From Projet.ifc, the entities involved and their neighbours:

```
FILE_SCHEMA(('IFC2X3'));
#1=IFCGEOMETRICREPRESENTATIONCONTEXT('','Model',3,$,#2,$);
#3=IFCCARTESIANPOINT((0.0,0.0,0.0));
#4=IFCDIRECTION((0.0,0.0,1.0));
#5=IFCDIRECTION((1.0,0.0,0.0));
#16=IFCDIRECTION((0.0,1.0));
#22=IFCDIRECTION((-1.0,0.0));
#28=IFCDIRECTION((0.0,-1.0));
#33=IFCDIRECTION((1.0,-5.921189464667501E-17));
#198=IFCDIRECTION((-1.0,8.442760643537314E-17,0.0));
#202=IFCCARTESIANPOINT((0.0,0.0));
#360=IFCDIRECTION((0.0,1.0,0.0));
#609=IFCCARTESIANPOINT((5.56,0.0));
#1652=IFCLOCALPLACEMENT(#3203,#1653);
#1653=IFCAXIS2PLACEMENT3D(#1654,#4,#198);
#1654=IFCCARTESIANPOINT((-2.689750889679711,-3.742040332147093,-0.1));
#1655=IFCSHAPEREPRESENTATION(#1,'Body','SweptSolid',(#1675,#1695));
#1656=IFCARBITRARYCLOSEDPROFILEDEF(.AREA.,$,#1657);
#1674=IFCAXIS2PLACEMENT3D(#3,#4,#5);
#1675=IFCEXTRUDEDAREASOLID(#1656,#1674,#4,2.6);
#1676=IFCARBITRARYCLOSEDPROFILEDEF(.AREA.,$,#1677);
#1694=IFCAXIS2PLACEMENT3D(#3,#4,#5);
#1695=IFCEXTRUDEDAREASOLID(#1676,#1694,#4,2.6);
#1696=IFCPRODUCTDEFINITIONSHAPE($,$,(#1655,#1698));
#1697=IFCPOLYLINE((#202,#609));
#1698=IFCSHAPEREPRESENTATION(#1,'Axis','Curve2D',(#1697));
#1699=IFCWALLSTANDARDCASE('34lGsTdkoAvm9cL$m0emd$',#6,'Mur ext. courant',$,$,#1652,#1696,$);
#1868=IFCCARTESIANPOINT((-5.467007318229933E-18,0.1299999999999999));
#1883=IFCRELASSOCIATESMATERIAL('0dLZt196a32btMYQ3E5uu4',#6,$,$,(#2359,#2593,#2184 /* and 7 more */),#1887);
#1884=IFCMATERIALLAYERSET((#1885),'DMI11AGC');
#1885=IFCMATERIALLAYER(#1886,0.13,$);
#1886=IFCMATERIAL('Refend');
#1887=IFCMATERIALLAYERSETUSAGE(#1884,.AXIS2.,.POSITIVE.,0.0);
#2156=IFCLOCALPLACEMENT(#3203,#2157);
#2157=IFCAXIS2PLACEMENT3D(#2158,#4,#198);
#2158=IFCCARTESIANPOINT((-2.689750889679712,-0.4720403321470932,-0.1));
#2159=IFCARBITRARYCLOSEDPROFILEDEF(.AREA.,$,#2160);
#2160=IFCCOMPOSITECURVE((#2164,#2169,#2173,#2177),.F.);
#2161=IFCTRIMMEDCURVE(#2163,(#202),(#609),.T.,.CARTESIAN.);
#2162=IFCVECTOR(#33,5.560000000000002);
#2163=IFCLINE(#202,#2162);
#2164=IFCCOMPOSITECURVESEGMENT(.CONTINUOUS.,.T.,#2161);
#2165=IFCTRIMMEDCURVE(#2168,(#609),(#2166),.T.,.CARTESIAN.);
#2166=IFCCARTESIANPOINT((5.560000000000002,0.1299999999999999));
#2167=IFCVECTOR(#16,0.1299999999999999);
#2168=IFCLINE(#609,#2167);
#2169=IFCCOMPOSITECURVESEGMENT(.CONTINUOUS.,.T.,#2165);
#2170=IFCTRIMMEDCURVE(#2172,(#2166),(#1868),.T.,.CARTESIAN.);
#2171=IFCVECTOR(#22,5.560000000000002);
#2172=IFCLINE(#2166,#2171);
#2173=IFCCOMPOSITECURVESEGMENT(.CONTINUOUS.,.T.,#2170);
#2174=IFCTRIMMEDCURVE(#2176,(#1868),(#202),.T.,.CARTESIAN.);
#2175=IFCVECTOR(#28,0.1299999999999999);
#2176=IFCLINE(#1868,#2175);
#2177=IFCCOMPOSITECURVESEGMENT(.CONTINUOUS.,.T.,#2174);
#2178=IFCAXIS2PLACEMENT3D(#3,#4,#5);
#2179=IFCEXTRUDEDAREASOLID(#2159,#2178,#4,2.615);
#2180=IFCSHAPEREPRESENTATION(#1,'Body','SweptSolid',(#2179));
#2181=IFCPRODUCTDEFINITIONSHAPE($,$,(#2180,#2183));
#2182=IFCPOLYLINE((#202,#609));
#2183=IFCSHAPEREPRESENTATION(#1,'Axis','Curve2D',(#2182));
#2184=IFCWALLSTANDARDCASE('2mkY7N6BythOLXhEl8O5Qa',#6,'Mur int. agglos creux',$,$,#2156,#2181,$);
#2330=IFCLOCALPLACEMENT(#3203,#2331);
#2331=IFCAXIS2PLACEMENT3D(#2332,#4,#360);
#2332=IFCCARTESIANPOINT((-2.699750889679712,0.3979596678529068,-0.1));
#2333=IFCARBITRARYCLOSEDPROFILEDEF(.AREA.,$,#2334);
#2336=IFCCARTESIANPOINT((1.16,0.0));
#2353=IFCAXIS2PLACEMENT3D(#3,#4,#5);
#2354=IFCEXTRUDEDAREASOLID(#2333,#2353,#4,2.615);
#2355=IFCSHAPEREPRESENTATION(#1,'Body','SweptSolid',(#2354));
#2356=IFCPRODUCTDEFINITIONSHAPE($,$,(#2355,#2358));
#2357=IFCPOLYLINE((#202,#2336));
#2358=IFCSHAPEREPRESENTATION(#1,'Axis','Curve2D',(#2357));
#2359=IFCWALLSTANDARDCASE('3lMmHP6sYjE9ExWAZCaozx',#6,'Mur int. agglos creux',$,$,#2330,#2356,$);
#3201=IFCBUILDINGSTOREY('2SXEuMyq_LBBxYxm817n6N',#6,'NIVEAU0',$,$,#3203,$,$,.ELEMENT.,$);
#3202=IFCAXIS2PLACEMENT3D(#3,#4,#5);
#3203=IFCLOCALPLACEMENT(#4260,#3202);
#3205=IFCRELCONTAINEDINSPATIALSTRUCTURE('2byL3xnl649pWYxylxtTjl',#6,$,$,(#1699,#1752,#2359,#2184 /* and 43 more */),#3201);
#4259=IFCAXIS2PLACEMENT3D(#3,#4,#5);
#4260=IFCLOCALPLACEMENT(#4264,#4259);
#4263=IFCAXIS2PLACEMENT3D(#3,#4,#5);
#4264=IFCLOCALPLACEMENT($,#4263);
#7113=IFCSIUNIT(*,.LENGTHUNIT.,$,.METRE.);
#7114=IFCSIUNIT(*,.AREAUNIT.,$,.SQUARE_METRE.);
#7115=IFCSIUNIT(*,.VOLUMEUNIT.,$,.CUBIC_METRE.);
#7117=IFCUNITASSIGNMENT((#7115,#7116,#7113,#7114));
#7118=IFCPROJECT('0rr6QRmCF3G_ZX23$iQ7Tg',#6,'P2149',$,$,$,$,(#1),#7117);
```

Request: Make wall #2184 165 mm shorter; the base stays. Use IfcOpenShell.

```python
import ifcopenshell
import ifcopenshell.geom
import ifcopenshell.util.shape
import ifcopenshell.util.unit

model = ifcopenshell.open("Projet.ifc")
unit_scale = ifcopenshell.util.unit.calculate_unit_scale(model)
settings = ifcopenshell.geom.settings()


def volume(element):
    """Net volume in cubic metres, openings subtracted."""
    shape = ifcopenshell.geom.create_shape(settings, element)
    return ifcopenshell.util.shape.get_volume(shape.geometry)


wall = model.by_guid("2mkY7N6BythOLXhEl8O5Qa")
before = volume(wall)

body = next(r for r in wall.Representation.Representations if r.RepresentationIdentifier == "Body")
solid = body.Items[0]
old_height = solid.Depth
solid.Depth -= 0.165 / unit_scale
after = volume(wall)

print(f"height {old_height:g} -> {solid.Depth:g}, volume {before:.3f} -> {after:.3f} m3")

model.write("Projet_edited.ifc")
```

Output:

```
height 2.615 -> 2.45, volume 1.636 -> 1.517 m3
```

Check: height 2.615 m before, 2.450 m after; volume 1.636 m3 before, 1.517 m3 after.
